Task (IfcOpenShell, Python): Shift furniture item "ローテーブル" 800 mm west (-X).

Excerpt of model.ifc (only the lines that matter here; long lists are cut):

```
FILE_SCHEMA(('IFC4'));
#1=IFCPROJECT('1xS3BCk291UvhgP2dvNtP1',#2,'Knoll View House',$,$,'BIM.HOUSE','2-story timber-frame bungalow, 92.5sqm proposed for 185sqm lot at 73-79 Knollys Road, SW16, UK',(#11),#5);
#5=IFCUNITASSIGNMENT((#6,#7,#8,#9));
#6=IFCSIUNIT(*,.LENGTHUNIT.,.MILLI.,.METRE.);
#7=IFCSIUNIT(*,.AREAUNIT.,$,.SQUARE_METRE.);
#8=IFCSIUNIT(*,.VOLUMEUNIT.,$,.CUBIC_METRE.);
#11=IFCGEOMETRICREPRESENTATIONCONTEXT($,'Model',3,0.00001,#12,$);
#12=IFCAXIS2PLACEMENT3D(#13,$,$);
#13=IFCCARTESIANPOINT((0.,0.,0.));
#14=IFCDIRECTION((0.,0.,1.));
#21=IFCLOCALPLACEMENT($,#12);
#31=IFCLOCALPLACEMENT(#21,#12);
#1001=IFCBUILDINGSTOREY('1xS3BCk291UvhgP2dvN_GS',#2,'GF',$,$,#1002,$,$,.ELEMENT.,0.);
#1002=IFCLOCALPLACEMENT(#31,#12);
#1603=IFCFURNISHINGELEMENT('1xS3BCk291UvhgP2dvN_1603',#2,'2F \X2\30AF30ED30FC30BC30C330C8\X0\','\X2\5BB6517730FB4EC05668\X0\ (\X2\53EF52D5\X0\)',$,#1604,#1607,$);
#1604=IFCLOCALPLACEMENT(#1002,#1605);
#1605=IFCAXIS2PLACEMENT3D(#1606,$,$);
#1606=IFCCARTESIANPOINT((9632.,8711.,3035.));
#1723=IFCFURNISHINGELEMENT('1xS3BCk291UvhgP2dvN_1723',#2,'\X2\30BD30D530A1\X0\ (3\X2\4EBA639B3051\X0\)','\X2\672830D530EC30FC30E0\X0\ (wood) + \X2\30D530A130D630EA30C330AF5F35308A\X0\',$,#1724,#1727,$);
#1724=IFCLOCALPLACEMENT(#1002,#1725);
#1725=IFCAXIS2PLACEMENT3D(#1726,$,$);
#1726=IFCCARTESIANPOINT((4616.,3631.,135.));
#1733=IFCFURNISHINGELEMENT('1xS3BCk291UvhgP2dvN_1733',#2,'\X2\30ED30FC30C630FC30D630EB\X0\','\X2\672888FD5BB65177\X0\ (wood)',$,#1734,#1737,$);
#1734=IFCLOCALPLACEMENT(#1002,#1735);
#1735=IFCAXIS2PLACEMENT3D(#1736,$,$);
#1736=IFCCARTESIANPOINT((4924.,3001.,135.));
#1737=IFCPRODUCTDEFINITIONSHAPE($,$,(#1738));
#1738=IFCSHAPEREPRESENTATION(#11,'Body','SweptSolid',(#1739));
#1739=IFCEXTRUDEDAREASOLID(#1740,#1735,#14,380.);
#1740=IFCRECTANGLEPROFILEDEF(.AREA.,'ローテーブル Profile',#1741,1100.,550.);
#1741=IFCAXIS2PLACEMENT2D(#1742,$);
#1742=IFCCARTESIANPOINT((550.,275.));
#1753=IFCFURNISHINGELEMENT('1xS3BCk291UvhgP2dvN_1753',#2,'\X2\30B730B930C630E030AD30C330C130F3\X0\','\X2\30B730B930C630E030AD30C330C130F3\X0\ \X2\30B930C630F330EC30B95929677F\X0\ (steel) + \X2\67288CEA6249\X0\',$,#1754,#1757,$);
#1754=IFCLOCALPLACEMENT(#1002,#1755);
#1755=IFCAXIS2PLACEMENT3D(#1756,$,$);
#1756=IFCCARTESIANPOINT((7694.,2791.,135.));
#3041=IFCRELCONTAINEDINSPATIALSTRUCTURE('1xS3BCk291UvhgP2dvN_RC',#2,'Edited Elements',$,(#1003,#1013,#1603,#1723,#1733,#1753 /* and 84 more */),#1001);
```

```python
import ifcopenshell
import ifcopenshell.api.geometry
import ifcopenshell.util.placement
import ifcopenshell.util.unit

model = ifcopenshell.open("model.ifc")
unit_scale = ifcopenshell.util.unit.calculate_unit_scale(model)

item = model.by_guid("1xS3BCk291UvhgP2dvN_1733")
matrix = ifcopenshell.util.placement.get_local_placement(item.ObjectPlacement)
matrix[0, 3] -= 0.8 / unit_scale
ifcopenshell.api.geometry.edit_object_placement(model, product=item, matrix=matrix, is_si=False)

print(ifcopenshell.util.placement.get_local_placement(item.ObjectPlacement).round(3) + 0.0)

model.write("model_rev.ifc")
```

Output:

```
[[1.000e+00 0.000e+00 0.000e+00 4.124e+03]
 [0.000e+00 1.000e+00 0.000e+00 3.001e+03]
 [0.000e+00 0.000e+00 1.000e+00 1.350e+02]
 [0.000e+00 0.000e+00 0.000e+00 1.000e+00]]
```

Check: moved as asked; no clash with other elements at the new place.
